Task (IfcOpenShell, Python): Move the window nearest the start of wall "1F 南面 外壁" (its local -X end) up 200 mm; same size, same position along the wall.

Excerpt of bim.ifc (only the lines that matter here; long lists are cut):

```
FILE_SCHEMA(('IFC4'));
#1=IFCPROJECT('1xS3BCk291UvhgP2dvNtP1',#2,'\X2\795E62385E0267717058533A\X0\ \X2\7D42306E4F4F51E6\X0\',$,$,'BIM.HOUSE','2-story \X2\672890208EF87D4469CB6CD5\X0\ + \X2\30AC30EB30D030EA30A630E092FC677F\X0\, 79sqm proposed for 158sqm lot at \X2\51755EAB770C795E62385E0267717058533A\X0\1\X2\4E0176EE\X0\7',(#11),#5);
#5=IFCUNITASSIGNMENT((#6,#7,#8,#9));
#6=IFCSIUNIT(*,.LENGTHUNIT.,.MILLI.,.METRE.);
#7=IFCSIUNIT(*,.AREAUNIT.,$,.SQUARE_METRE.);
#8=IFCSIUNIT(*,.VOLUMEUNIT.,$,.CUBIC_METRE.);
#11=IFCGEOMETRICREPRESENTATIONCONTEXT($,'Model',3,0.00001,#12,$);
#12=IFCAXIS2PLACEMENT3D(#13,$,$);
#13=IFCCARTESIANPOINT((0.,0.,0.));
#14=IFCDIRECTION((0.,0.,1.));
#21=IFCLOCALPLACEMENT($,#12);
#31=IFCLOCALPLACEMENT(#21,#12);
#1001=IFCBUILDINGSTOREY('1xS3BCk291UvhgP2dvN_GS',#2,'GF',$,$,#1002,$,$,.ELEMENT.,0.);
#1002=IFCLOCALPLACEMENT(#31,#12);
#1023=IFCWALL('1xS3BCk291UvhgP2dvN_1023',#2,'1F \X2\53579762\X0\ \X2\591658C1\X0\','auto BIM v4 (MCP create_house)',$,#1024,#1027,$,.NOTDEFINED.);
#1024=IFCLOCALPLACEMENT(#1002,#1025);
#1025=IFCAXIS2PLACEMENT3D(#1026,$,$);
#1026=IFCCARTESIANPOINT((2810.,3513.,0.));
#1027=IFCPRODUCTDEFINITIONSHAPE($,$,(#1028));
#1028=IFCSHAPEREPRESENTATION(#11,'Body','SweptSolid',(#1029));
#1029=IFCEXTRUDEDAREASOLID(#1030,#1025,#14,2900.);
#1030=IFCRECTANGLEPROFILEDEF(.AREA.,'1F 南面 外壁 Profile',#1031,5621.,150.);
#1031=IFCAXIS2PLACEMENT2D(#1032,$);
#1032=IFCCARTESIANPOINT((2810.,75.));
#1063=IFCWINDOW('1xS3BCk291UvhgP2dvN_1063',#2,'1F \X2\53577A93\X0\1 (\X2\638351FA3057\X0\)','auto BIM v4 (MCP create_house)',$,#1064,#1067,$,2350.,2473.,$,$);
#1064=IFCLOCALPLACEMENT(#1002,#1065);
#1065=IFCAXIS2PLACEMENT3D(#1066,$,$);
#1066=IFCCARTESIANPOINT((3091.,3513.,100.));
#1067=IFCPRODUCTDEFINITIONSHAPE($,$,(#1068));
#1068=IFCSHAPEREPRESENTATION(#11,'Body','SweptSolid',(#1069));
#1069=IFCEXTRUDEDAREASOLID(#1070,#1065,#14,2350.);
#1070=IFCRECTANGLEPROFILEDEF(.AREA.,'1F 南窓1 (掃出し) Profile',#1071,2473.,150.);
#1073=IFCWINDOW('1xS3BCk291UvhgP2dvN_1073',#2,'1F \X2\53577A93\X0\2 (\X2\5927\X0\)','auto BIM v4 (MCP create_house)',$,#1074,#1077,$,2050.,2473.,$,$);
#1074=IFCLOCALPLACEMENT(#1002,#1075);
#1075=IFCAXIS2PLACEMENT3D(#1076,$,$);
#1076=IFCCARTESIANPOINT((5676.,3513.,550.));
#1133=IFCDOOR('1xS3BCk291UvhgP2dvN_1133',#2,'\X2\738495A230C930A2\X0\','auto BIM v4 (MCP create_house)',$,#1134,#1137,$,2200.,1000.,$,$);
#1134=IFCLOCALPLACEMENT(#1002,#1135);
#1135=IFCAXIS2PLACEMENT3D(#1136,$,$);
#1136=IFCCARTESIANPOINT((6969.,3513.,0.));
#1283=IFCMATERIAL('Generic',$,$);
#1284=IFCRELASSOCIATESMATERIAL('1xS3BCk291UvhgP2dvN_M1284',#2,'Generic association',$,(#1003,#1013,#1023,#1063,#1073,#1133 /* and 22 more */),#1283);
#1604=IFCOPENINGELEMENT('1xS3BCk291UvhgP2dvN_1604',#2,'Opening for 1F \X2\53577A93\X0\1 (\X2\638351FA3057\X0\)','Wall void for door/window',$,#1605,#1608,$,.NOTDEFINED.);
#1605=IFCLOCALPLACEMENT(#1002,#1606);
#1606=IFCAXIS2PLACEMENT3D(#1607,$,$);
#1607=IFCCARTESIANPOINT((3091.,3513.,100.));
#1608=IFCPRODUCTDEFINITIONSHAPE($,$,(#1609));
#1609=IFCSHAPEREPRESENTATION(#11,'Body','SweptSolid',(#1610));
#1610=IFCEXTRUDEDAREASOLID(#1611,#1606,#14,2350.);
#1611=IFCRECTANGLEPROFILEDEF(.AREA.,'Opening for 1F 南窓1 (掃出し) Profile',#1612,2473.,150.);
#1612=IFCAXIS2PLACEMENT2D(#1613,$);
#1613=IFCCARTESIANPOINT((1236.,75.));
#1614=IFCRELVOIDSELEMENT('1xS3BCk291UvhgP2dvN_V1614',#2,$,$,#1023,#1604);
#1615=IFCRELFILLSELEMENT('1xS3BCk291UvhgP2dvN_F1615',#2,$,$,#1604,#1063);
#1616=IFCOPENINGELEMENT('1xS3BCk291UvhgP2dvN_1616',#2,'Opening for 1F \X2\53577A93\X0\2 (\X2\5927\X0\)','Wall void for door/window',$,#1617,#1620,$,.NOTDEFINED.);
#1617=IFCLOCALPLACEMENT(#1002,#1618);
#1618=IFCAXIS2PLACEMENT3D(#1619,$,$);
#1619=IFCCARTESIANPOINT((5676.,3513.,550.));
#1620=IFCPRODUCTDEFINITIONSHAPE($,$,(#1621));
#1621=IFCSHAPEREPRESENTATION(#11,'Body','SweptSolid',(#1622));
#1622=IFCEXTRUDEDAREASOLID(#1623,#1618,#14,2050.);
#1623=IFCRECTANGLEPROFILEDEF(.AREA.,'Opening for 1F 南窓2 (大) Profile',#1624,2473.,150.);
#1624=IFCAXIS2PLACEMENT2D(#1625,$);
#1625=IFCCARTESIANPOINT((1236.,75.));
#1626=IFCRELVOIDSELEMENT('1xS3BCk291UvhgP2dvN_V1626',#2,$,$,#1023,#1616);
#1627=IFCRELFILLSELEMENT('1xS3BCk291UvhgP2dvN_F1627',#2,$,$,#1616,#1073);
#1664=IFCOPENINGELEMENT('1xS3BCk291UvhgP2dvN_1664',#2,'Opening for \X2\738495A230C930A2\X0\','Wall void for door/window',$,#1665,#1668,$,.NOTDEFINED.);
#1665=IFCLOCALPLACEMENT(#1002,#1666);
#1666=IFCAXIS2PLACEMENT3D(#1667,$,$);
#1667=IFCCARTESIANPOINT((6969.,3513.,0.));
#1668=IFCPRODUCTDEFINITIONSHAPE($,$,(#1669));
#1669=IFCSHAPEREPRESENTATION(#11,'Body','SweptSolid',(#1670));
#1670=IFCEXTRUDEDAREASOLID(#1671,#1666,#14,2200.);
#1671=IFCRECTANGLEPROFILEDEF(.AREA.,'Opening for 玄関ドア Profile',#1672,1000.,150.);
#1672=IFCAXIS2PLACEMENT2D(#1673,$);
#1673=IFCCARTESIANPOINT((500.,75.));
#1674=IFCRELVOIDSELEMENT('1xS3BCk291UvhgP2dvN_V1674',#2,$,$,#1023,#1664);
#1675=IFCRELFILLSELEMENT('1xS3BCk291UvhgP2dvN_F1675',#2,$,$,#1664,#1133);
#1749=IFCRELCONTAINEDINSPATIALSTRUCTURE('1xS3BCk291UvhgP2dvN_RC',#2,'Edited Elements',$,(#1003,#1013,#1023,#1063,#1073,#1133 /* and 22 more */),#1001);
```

```python
import numpy as np
import ifcopenshell
import ifcopenshell.api.geometry
import ifcopenshell.util.placement
import ifcopenshell.util.unit

model = ifcopenshell.open("bim.ifc")
unit_scale = ifcopenshell.util.unit.calculate_unit_scale(model)

window = model.by_guid("1xS3BCk291UvhgP2dvN_1063")
opening = window.FillsVoids[0].RelatingOpeningElement
dz = 200.0

shift = np.array([0.0, 0.0, dz])
# The window is not placed relative to its opening, so move both.
for product in (opening, window):
    matrix = ifcopenshell.util.placement.get_local_placement(product.ObjectPlacement)
    matrix[:3, 3] += shift
    ifcopenshell.api.geometry.edit_object_placement(model, product=product, matrix=matrix, is_si=False)

print(f"moved by {dz * unit_scale:+.3f} m")

model.write("bim_edited.ifc")
```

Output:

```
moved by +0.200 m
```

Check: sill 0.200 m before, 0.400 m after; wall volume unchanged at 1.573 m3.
